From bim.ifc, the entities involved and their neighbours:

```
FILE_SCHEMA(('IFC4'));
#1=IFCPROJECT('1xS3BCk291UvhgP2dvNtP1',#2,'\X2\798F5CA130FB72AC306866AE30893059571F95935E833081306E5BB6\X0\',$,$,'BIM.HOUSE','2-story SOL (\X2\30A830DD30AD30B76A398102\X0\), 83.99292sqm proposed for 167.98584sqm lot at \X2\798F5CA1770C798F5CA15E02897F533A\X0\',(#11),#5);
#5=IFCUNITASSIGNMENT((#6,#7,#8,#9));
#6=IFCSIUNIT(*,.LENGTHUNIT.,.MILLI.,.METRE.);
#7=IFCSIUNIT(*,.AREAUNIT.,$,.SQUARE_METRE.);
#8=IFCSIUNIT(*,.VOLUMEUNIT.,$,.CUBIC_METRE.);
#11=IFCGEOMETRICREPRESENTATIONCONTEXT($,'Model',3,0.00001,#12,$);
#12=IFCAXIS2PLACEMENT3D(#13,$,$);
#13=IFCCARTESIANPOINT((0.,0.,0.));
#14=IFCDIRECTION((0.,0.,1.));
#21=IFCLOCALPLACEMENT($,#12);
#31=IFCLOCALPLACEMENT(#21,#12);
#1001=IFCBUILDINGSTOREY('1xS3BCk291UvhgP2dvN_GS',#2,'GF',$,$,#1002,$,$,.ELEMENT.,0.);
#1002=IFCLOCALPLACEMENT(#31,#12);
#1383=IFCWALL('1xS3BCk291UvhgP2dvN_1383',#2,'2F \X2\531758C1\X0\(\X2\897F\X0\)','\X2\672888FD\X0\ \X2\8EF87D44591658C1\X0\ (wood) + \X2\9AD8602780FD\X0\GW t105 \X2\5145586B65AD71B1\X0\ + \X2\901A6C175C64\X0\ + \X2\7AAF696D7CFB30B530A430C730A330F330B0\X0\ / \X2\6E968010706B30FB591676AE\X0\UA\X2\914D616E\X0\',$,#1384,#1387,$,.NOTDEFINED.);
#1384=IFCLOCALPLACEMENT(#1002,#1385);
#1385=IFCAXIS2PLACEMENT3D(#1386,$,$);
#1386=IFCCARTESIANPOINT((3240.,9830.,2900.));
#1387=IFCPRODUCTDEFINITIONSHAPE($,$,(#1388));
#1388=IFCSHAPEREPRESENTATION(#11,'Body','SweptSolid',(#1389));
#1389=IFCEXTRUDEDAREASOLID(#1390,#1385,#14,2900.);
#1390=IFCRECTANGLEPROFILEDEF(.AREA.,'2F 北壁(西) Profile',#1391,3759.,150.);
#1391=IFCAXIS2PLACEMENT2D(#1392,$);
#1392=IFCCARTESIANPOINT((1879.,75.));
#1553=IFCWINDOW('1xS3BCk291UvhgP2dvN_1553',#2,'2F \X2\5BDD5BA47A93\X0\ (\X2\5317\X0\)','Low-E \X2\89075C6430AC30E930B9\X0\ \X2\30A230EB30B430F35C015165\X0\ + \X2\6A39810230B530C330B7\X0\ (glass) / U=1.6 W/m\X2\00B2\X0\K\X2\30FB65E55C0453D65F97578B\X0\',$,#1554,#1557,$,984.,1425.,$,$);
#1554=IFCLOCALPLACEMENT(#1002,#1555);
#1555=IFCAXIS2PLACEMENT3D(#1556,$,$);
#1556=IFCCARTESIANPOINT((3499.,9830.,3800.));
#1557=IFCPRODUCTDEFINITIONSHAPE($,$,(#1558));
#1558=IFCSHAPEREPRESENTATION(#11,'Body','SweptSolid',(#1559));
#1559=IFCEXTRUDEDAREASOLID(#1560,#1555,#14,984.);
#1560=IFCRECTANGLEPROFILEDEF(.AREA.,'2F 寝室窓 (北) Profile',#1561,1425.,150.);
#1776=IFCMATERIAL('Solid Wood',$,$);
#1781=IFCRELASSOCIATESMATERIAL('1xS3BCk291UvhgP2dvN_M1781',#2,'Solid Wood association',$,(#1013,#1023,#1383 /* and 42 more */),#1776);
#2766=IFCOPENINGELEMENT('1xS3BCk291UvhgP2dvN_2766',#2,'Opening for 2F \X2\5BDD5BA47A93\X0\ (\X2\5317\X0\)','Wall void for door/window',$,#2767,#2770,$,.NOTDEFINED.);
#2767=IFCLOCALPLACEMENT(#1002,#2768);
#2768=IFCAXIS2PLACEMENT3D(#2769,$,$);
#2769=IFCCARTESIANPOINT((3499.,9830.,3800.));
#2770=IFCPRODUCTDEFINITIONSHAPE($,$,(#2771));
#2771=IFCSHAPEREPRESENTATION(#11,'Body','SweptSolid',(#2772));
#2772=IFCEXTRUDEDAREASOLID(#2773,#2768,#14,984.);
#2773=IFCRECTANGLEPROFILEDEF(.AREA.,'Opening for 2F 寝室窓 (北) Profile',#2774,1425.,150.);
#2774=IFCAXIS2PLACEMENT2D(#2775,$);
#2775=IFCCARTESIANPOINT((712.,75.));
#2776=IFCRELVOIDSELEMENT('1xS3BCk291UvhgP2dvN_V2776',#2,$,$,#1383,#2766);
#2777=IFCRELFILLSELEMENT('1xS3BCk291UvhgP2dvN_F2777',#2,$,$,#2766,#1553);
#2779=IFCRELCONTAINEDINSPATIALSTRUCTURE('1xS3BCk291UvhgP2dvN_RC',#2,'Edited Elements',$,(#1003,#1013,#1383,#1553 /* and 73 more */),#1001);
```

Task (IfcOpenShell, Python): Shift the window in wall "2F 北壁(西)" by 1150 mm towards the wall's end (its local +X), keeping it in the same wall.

```python
import ifcopenshell
import ifcopenshell.api.geometry
import ifcopenshell.util.placement
import ifcopenshell.util.unit

model = ifcopenshell.open("bim.ifc")
unit_scale = ifcopenshell.util.unit.calculate_unit_scale(model)

window = model.by_guid("1xS3BCk291UvhgP2dvN_1553")
opening = window.FillsVoids[0].RelatingOpeningElement
wall = opening.VoidsElements[0].RelatingBuildingElement

wall_matrix = ifcopenshell.util.placement.get_local_placement(wall.ObjectPlacement)
shift = wall_matrix[:3, 0] * 1.15 / unit_scale
before = ifcopenshell.util.placement.get_local_placement(window.ObjectPlacement)[:3, 3].copy()

# The window is not placed relative to its opening, so move both.
for product in (opening, window):
    matrix = ifcopenshell.util.placement.get_local_placement(product.ObjectPlacement)
    matrix[:3, 3] += shift
    ifcopenshell.api.geometry.edit_object_placement(model, product=product, matrix=matrix, is_si=False)

after = ifcopenshell.util.placement.get_local_placement(window.ObjectPlacement)[:3, 3]
print("window moved by", (after - before).round(3) + 0.0)

model.write("bim_updated.ifc")
```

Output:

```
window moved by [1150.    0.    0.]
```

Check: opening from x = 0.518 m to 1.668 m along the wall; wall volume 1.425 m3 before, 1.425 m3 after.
